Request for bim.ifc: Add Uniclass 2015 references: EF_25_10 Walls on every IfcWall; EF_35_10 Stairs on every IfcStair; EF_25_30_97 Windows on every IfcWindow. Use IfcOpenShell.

First a look at what the model holds.

```python
import ifcopenshell

model = ifcopenshell.open("bim.ifc")
print(model.schema)
print("classifications:", [c.Name for c in model.by_type("IfcClassification")])
for ifc_class in ("IfcDoor", "IfcRoof", "IfcStair", "IfcWall", "IfcWindow"):
    print(ifc_class, len(model.by_type(ifc_class)))
```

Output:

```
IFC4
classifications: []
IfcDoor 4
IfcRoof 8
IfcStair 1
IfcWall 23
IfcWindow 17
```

```python
import ifcopenshell
import ifcopenshell.api.classification

model = ifcopenshell.open("bim.ifc")

system = ifcopenshell.api.classification.add_classification(model, classification="Uniclass 2015")

codes = {
    "IfcWall": ("EF_25_10", "Walls"),
    "IfcStair": ("EF_35_10", "Stairs"),
    "IfcWindow": ("EF_25_30_97", "Windows"),
}
for ifc_class, (code, name) in codes.items():
    products = model.by_type(ifc_class)
    ifcopenshell.api.classification.add_reference(
        model, products=products, classification=system, identification=code, name=name
    )
    print(code, len(products))

model.write("bim-out.ifc")
```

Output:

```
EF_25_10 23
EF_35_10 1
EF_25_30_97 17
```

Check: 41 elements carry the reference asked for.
